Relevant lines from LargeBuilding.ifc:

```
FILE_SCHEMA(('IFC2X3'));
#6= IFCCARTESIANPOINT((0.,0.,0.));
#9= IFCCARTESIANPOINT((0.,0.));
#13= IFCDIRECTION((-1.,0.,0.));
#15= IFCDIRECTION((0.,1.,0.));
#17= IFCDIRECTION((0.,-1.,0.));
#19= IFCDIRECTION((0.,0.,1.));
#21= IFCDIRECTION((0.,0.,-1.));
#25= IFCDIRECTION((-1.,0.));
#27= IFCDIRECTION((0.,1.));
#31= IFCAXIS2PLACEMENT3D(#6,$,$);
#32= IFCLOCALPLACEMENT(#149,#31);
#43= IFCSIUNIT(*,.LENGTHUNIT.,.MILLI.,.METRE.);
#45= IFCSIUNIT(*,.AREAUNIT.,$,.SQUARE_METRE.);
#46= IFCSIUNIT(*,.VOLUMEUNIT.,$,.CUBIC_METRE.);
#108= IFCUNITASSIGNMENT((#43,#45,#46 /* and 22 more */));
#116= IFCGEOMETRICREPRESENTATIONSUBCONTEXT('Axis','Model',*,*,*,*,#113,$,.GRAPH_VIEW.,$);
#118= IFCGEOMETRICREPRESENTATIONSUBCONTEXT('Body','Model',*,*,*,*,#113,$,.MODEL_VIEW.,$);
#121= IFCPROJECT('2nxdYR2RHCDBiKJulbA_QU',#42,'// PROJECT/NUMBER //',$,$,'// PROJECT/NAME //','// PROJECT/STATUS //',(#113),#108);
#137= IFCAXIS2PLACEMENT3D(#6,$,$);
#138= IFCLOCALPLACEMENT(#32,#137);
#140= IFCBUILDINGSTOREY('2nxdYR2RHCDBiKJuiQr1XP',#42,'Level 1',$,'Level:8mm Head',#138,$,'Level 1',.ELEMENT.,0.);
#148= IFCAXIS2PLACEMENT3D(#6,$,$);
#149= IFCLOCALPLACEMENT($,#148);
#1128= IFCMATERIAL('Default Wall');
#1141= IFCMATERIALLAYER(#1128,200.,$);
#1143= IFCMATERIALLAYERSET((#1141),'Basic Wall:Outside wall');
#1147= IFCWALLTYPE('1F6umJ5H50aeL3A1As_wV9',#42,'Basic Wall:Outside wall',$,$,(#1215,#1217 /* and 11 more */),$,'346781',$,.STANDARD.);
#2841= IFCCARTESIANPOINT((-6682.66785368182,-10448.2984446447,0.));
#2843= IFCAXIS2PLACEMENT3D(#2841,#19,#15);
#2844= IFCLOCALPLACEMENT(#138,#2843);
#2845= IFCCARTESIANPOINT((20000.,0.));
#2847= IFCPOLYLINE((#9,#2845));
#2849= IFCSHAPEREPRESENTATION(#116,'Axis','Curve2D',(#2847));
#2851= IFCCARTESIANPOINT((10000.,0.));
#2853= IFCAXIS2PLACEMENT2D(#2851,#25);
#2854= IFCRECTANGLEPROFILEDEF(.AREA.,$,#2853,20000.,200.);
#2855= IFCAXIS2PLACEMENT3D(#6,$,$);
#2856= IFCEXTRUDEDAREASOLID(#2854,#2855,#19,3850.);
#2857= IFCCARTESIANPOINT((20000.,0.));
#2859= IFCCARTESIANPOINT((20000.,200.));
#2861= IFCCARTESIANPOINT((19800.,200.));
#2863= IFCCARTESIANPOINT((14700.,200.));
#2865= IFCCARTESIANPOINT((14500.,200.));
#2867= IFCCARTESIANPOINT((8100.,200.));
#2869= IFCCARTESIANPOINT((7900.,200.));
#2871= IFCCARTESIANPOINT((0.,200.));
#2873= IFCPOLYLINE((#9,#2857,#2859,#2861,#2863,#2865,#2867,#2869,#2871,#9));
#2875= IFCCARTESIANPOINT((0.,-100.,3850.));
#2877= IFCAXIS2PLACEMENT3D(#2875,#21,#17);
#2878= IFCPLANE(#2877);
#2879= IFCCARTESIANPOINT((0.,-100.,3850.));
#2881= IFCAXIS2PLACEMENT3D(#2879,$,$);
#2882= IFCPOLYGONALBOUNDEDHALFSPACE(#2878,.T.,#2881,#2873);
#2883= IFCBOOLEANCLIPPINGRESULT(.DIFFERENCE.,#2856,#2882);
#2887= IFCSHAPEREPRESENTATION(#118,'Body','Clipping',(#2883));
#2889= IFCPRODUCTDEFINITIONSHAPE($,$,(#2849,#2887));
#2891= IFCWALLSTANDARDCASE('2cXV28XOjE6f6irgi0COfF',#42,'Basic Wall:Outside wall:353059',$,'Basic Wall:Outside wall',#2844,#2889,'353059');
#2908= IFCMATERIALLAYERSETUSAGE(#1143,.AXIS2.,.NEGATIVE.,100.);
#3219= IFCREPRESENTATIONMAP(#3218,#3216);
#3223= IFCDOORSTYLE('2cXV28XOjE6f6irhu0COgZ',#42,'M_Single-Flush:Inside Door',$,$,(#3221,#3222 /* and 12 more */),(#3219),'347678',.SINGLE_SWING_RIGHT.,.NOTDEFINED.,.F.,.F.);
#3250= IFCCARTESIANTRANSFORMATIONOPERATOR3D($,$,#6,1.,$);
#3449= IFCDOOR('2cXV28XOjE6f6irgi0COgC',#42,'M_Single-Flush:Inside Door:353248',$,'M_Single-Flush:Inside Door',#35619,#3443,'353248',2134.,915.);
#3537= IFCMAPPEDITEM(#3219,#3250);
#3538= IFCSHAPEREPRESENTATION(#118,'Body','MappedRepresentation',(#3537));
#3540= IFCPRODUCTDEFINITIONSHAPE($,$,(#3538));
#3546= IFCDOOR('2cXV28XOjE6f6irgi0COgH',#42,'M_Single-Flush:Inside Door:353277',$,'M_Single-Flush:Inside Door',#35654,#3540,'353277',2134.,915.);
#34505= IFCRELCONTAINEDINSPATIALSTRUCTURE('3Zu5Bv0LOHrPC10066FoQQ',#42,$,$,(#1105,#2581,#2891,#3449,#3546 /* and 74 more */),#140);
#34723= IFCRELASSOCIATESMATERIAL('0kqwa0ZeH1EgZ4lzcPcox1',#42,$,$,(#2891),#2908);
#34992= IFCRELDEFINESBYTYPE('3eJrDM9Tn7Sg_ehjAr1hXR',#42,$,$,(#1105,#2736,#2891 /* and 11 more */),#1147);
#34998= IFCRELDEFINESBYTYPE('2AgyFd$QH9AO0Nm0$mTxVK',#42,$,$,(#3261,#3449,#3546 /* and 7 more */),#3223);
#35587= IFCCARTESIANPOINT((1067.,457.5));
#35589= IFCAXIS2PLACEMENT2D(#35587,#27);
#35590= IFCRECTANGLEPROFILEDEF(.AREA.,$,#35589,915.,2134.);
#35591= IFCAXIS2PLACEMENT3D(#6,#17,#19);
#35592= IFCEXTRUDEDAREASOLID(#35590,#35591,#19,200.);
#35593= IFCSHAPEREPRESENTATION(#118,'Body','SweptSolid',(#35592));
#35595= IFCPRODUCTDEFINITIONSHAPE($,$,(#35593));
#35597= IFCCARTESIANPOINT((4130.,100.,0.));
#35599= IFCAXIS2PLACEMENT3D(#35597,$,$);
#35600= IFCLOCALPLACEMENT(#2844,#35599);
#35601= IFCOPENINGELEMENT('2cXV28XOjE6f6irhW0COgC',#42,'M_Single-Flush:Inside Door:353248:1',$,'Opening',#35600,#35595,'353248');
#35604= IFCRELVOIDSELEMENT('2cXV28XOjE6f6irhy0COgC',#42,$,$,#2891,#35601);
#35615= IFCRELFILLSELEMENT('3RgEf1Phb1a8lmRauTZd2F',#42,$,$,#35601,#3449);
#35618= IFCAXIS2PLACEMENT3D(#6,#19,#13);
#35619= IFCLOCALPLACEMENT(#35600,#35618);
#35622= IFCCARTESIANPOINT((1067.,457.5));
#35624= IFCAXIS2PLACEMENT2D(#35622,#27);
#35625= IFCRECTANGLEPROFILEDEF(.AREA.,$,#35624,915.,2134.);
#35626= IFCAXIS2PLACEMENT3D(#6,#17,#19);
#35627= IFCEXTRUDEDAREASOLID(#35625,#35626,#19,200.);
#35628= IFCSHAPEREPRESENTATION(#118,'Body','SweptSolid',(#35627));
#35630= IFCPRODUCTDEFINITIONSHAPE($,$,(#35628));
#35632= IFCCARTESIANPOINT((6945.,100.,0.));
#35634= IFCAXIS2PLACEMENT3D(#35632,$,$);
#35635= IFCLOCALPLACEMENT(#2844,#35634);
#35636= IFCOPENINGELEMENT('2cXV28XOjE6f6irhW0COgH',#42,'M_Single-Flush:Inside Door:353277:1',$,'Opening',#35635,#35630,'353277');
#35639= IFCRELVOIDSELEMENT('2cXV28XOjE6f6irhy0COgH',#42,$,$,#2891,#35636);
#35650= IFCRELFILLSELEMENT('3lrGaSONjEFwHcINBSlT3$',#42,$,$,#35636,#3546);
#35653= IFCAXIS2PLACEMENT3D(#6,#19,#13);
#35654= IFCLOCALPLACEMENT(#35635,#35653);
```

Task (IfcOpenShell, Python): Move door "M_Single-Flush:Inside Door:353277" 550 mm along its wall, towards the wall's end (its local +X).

```python
import ifcopenshell
import ifcopenshell.api.geometry
import ifcopenshell.util.placement
import ifcopenshell.util.unit

model = ifcopenshell.open("LargeBuilding.ifc")
unit_scale = ifcopenshell.util.unit.calculate_unit_scale(model)

door = model.by_guid("2cXV28XOjE6f6irgi0COgH")
opening = door.FillsVoids[0].RelatingOpeningElement
wall = opening.VoidsElements[0].RelatingBuildingElement

wall_matrix = ifcopenshell.util.placement.get_local_placement(wall.ObjectPlacement)
shift = wall_matrix[:3, 0] * 0.55 / unit_scale
before = ifcopenshell.util.placement.get_local_placement(door.ObjectPlacement)[:3, 3].copy()

# The door is placed relative to its opening, so it follows when the opening moves.
matrix = ifcopenshell.util.placement.get_local_placement(opening.ObjectPlacement)
matrix[:3, 3] += shift
ifcopenshell.api.geometry.edit_object_placement(
    model, product=opening, matrix=matrix, is_si=False, should_transform_children=True
)

after = ifcopenshell.util.placement.get_local_placement(door.ObjectPlacement)[:3, 3]
print("door moved by", (after - before).round(3) + 0.0)

model.write("LargeBuilding_updated.ifc")
```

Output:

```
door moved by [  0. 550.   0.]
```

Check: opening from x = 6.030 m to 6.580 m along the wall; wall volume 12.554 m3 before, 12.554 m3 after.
